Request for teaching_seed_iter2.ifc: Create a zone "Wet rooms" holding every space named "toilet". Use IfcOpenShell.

First a look at what the model holds.

```python
import ifcopenshell

model = ifcopenshell.open("teaching_seed_iter2.ifc")
print(model.schema)
seen = {}
for space in model.by_type("IfcSpace"):
    seen[space.LongName] = seen.get(space.LongName, 0) + 1
for name, count in sorted(seen.items(), key=str):
    print(count, "x", name)
print("zones:", [z.Name for z in model.by_type("IfcZone")][:20])
```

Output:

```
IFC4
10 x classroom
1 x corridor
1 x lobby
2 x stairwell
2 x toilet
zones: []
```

```python
import ifcopenshell
import ifcopenshell.api.group
import ifcopenshell.api.root

model = ifcopenshell.open("teaching_seed_iter2.ifc")

names = {"toilet"}
spaces = [s for s in model.by_type("IfcSpace") if s.LongName in names]

zone = ifcopenshell.api.root.create_entity(model, ifc_class="IfcZone", name="Wet rooms")
ifcopenshell.api.group.assign_group(model, products=spaces, group=zone)
print(len(spaces), "spaces in", zone.Name)

model.write("teaching_seed_iter2_v2.ifc")
```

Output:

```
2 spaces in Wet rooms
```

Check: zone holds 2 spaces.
